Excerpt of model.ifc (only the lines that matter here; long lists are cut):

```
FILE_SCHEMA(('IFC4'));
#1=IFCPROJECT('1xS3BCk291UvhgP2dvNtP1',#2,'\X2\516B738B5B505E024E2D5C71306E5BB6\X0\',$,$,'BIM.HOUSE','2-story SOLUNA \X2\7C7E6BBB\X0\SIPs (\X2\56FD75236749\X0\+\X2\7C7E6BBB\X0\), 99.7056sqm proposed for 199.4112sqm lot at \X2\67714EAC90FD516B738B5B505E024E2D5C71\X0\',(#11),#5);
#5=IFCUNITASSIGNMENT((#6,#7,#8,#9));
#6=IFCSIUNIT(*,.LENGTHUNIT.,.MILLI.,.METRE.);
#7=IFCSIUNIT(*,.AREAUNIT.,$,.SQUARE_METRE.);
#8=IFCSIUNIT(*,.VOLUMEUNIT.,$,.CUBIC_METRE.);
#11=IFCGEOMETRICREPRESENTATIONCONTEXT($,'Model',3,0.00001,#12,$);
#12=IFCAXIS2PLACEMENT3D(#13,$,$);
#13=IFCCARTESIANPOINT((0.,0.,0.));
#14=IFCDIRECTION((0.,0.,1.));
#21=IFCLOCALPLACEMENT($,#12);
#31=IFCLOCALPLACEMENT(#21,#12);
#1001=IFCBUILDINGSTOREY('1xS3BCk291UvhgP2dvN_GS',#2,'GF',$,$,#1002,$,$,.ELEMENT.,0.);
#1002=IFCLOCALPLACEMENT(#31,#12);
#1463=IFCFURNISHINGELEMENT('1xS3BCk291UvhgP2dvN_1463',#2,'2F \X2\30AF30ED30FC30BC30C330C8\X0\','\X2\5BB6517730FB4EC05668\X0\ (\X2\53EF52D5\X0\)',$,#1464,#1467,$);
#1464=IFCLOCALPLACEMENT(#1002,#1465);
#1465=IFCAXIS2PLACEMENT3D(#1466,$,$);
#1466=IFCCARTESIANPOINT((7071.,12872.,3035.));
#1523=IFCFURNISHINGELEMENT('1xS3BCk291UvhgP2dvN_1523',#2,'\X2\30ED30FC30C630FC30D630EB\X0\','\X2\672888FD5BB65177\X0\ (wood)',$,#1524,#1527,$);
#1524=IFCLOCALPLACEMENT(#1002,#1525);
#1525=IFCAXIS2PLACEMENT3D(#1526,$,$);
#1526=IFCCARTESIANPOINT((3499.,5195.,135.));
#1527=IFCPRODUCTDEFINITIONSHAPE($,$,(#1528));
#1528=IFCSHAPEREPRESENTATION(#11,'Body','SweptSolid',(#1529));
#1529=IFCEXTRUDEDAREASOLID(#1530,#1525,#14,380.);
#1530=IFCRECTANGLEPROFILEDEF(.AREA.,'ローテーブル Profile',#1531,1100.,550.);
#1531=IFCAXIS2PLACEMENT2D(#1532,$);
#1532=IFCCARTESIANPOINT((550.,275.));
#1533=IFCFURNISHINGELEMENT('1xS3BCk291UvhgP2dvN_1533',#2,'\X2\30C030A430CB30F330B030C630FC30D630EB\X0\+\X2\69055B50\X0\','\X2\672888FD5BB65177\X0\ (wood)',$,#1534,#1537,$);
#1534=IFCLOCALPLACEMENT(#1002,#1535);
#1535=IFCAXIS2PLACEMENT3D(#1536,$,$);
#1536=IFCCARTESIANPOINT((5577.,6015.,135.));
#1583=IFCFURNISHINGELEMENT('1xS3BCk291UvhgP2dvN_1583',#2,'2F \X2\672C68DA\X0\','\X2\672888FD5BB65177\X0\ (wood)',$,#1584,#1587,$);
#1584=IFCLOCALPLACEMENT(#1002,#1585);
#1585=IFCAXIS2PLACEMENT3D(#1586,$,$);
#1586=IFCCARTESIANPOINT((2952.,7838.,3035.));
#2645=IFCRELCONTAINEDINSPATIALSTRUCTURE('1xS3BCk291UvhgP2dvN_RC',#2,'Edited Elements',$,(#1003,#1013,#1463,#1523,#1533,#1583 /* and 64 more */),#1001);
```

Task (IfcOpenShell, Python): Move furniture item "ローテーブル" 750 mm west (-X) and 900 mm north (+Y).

```python
import ifcopenshell
import ifcopenshell.api.geometry
import ifcopenshell.util.placement

model = ifcopenshell.open("model.ifc")

item = model.by_guid("1xS3BCk291UvhgP2dvN_1523")
matrix = ifcopenshell.util.placement.get_local_placement(item.ObjectPlacement)
matrix[0, 3] -= 750.0
matrix[1, 3] += 900.0
ifcopenshell.api.geometry.edit_object_placement(model, product=item, matrix=matrix, is_si=False)

print(ifcopenshell.util.placement.get_local_placement(item.ObjectPlacement).round(3) + 0.0)

model.write("model_v2.ifc")
```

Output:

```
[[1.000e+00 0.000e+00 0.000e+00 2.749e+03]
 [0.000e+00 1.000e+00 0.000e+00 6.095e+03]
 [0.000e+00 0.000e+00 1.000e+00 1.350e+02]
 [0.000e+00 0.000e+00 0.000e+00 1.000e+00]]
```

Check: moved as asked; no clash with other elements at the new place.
